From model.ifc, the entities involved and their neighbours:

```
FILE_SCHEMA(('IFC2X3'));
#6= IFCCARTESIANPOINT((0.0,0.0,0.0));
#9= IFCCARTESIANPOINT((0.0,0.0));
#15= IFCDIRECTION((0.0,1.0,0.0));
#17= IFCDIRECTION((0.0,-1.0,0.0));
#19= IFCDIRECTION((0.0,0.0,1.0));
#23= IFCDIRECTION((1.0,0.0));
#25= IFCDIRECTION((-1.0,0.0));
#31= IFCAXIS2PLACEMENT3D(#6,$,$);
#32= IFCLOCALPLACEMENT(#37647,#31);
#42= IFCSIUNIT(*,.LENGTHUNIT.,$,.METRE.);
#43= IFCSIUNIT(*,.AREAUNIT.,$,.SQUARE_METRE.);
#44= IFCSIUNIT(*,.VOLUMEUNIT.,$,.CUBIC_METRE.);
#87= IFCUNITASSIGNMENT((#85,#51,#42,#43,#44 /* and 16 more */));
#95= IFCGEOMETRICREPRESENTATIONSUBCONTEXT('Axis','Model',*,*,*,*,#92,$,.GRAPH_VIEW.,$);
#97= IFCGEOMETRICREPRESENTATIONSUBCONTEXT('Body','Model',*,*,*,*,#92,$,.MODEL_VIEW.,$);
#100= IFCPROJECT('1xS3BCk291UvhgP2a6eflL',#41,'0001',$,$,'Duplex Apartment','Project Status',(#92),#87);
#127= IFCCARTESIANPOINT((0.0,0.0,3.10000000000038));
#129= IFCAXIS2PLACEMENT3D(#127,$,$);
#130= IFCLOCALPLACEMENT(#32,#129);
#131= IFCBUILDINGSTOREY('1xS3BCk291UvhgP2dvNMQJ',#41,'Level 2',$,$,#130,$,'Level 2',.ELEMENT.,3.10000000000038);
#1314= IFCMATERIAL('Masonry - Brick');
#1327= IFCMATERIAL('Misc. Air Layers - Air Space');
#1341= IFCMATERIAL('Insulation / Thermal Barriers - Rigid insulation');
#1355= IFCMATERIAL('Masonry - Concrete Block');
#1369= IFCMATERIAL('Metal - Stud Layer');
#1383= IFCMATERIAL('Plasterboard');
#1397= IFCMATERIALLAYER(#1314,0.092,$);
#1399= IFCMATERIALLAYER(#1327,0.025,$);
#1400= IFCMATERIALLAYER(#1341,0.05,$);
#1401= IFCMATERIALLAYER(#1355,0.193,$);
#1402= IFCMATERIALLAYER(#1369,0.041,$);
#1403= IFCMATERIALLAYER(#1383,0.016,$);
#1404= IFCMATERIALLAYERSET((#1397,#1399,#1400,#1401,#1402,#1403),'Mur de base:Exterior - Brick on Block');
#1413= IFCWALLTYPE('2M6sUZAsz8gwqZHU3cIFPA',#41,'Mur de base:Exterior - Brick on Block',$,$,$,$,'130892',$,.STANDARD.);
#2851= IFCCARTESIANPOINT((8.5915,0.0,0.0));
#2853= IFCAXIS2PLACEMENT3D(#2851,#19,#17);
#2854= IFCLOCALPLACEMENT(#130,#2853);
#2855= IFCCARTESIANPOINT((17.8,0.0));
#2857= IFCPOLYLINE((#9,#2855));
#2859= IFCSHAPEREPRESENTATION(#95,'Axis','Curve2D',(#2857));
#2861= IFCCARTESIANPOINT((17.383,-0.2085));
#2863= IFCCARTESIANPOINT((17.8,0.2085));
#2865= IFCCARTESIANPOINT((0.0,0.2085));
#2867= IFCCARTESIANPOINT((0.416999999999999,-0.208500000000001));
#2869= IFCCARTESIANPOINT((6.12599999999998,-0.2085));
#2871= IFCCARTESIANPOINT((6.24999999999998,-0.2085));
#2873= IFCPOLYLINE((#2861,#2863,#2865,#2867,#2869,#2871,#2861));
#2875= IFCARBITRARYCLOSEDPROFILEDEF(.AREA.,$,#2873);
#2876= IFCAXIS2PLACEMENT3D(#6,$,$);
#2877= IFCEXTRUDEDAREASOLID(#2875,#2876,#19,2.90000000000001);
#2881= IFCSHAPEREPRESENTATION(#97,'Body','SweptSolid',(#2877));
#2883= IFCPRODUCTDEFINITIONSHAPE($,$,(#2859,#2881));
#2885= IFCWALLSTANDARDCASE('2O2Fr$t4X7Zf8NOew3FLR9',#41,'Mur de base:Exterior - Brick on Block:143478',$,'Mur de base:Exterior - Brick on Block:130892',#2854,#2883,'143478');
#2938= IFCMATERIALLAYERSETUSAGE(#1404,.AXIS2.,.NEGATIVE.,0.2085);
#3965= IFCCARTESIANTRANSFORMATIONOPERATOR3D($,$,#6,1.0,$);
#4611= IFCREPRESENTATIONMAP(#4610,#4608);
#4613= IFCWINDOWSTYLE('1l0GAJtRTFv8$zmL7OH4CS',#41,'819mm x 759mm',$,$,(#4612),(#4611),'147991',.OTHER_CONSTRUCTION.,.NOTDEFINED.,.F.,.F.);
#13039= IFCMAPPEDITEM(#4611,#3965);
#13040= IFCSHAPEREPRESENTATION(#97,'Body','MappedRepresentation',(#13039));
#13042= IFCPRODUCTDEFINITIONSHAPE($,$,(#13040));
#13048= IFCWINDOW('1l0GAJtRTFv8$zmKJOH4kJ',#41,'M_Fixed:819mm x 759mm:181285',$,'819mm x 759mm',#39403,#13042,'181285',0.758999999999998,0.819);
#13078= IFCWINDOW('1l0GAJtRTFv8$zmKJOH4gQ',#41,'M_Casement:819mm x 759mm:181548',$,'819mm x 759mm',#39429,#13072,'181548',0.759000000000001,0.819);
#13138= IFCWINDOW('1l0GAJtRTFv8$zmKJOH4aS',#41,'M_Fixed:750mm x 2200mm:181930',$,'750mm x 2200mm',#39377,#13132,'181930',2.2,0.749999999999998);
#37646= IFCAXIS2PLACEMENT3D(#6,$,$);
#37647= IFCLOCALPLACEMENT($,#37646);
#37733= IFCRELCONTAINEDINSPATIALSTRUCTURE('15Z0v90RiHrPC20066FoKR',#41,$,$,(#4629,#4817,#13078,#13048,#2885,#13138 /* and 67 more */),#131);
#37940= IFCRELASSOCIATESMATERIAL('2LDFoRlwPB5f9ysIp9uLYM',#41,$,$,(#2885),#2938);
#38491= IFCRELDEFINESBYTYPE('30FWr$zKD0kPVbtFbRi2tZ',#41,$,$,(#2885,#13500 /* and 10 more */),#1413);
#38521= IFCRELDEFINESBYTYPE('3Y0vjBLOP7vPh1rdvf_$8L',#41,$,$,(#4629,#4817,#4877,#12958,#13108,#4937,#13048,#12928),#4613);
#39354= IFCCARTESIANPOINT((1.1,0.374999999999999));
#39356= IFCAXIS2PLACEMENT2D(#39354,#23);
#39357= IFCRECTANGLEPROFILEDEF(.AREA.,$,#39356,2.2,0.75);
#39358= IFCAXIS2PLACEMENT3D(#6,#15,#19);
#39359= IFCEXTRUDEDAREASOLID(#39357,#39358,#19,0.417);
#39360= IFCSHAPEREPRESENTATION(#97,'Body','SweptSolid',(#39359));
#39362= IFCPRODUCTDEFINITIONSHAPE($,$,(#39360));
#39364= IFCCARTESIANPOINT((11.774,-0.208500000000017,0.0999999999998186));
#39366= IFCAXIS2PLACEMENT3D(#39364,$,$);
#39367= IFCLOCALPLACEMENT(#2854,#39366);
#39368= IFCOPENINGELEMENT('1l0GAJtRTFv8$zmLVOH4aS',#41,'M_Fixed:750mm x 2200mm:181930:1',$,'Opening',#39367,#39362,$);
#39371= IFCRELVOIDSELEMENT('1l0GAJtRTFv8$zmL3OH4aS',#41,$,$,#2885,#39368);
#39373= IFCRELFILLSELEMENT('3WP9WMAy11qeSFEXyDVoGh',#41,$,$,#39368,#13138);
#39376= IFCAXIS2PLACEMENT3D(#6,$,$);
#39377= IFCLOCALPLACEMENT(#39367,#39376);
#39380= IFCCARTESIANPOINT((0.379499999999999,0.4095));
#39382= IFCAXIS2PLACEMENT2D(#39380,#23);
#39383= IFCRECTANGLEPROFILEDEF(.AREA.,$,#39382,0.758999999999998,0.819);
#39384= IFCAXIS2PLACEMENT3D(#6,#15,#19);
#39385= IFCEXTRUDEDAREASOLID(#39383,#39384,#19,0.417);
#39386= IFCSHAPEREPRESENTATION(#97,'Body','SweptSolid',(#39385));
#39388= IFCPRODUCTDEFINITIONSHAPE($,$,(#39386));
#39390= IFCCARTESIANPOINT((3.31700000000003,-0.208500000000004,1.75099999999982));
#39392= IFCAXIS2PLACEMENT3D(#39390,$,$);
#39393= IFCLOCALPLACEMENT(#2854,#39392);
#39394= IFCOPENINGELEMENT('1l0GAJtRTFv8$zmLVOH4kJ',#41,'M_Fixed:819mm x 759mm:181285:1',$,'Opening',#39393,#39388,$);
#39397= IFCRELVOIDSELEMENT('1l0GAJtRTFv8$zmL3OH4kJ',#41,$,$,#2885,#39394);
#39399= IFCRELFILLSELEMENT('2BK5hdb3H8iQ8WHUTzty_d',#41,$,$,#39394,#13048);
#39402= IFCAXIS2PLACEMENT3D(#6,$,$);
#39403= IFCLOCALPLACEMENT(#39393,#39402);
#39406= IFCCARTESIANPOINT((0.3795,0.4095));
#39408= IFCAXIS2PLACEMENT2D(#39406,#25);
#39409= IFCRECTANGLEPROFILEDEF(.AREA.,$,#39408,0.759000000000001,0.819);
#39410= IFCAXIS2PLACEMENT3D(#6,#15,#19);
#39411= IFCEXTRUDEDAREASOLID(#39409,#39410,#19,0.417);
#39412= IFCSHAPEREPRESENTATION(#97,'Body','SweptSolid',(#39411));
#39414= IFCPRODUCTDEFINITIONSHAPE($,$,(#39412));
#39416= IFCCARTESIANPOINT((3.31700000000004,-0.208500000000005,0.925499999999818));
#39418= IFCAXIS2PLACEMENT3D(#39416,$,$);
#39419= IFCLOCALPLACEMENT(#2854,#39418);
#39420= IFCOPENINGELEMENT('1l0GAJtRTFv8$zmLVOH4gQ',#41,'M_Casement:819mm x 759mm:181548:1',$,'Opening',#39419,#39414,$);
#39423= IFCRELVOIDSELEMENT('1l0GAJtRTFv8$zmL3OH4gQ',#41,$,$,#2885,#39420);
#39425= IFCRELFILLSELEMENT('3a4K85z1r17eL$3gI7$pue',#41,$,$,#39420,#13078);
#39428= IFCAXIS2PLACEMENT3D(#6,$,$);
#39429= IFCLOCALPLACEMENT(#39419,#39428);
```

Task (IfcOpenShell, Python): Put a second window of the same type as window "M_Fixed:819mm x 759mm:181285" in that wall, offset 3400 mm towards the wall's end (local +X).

```python
import ifcopenshell
import ifcopenshell.api.feature
import ifcopenshell.api.geometry
import ifcopenshell.api.root
import ifcopenshell.geom
import ifcopenshell.util.element
import ifcopenshell.util.placement
import ifcopenshell.util.shape
import ifcopenshell.util.unit

model = ifcopenshell.open("model.ifc")
unit_scale = ifcopenshell.util.unit.calculate_unit_scale(model)
settings = ifcopenshell.geom.settings()


def volume(element):
    """Net volume in cubic metres, openings subtracted."""
    shape = ifcopenshell.geom.create_shape(settings, element)
    return ifcopenshell.util.shape.get_volume(shape.geometry)


def reuse_history(source, copy):
    """copy_class also copies each property set's owner history, people and application; keep the originals."""
    for rel in copy.IsDefinedBy:
        if rel.is_a("IfcRelDefinesByProperties") and (history := rel.RelatingPropertyDefinition.OwnerHistory):
            rel.RelatingPropertyDefinition.OwnerHistory = source.OwnerHistory
            ifcopenshell.util.element.remove_deep2(model, history)


window = model.by_guid("1l0GAJtRTFv8$zmKJOH4kJ")
opening = window.FillsVoids[0].RelatingOpeningElement
wall = opening.VoidsElements[0].RelatingBuildingElement
before = volume(wall)
shift = ifcopenshell.util.placement.get_local_placement(wall.ObjectPlacement)[:3, 0] * 3.4 / unit_scale

# copy_class copies the void relationship, type, container and properties, but no geometry.
new_opening = ifcopenshell.api.root.copy_class(model, product=opening)
new_opening.Representation = ifcopenshell.util.element.copy_deep(
    model, opening.Representation, exclude=["IfcGeometricRepresentationContext", "IfcRepresentationMap"]
)
new_opening.Name = "M_Fixed:819mm x 759mm"
new_window = ifcopenshell.api.root.copy_class(model, product=window)
new_window.Representation = ifcopenshell.util.element.copy_deep(
    model, window.Representation, exclude=["IfcGeometricRepresentationContext", "IfcRepresentationMap"]
)
new_window.Name = "M_Fixed:819mm x 759mm"
new_window.Tag = None
reuse_history(window, new_window)
fills = ifcopenshell.api.feature.add_filling(model, opening=new_opening, element=new_window)
fills.OwnerHistory = new_window.OwnerHistory  # required in IFC2X3

for old, new in ((opening, new_opening), (window, new_window)):
    matrix = ifcopenshell.util.placement.get_local_placement(old.ObjectPlacement)
    matrix[:3, 3] += shift
    ifcopenshell.api.geometry.edit_object_placement(model, product=new, matrix=matrix, is_si=False)

after = volume(wall)

print(f"wall volume {before:.3f} -> {after:.3f} m3")

model.write("model_v2.ifc")
```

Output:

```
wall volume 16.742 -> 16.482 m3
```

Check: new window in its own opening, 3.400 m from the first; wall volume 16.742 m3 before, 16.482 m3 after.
